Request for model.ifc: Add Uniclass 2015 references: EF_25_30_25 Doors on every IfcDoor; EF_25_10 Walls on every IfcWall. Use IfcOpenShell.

First a look at what the model holds.

```python
import ifcopenshell

model = ifcopenshell.open("model.ifc")
print(model.schema)
print("classifications:", [c.Name for c in model.by_type("IfcClassification")])
for ifc_class in ("IfcDoor", "IfcRoof", "IfcStair", "IfcWall", "IfcWindow"):
    print(ifc_class, len(model.by_type(ifc_class)))
```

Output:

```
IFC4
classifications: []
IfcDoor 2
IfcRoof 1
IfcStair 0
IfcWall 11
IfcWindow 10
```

```python
import ifcopenshell
import ifcopenshell.api.classification

model = ifcopenshell.open("model.ifc")

system = ifcopenshell.api.classification.add_classification(model, classification="Uniclass 2015")

codes = {
    "IfcDoor": ("EF_25_30_25", "Doors"),
    "IfcWall": ("EF_25_10", "Walls"),
}
for ifc_class, (code, name) in codes.items():
    products = model.by_type(ifc_class)
    ifcopenshell.api.classification.add_reference(
        model, products=products, classification=system, identification=code, name=name
    )
    print(code, len(products))

model.write("model_v2.ifc")
```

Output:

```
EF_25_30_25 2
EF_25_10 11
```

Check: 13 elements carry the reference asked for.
